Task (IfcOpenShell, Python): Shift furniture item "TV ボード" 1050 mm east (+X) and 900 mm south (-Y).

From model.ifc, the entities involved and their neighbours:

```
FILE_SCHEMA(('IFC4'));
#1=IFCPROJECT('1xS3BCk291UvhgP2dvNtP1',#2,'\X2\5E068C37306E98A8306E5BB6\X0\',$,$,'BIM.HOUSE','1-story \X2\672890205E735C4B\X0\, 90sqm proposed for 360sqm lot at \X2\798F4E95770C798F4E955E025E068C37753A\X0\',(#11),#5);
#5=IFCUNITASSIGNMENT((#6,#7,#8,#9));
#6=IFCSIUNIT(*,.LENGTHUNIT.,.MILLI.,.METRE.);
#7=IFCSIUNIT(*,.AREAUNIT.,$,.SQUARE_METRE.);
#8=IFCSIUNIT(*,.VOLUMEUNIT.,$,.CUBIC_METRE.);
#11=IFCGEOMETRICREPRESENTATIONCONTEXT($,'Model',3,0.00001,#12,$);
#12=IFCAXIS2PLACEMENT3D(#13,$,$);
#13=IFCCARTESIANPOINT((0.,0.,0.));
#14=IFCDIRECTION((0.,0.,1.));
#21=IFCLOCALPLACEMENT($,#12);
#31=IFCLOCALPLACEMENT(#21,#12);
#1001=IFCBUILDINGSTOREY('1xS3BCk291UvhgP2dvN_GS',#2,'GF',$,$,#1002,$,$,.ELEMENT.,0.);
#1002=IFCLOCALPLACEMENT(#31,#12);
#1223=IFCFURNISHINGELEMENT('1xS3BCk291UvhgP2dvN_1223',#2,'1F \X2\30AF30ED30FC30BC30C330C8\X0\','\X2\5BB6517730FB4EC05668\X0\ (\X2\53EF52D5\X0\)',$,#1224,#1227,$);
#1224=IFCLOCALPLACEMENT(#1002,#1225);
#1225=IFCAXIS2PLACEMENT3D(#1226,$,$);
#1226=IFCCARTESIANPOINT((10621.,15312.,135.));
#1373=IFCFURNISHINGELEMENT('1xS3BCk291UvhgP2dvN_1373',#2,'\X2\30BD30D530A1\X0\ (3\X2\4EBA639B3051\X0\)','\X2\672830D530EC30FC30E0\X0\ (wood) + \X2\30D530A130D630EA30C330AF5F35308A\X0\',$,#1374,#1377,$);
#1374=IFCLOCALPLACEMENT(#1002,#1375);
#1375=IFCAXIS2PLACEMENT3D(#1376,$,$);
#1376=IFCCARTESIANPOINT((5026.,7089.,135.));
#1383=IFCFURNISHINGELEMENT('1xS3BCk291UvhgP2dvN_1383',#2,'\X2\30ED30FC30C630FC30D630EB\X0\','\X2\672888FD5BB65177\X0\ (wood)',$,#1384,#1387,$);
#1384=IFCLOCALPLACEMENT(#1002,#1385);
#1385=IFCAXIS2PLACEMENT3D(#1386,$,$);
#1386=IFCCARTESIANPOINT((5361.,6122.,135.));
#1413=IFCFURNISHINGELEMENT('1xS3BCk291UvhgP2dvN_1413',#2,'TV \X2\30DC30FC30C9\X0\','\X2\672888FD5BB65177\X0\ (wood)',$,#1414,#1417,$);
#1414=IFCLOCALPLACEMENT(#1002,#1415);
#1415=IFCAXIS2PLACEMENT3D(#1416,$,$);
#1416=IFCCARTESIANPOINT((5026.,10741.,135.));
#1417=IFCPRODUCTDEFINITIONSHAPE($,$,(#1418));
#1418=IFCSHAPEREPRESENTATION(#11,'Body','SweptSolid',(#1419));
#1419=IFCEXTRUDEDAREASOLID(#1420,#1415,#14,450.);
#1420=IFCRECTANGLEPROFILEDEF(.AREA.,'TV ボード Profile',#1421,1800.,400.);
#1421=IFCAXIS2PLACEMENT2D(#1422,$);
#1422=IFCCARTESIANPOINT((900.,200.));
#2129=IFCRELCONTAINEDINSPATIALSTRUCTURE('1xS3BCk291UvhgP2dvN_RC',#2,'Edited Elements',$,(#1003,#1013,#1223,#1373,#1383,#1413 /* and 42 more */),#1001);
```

```python
import ifcopenshell
import ifcopenshell.api.geometry
import ifcopenshell.util.placement

model = ifcopenshell.open("model.ifc")

item = model.by_guid("1xS3BCk291UvhgP2dvN_1413")
matrix = ifcopenshell.util.placement.get_local_placement(item.ObjectPlacement)
matrix[0, 3] += 1050.0
matrix[1, 3] -= 900.0
ifcopenshell.api.geometry.edit_object_placement(model, product=item, matrix=matrix, is_si=False)

print(ifcopenshell.util.placement.get_local_placement(item.ObjectPlacement).round(3) + 0.0)

model.write("model_rev.ifc")
```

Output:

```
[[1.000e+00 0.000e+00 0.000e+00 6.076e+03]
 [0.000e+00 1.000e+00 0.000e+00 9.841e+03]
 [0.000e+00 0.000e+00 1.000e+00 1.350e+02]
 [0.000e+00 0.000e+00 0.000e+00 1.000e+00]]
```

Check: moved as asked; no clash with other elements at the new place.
